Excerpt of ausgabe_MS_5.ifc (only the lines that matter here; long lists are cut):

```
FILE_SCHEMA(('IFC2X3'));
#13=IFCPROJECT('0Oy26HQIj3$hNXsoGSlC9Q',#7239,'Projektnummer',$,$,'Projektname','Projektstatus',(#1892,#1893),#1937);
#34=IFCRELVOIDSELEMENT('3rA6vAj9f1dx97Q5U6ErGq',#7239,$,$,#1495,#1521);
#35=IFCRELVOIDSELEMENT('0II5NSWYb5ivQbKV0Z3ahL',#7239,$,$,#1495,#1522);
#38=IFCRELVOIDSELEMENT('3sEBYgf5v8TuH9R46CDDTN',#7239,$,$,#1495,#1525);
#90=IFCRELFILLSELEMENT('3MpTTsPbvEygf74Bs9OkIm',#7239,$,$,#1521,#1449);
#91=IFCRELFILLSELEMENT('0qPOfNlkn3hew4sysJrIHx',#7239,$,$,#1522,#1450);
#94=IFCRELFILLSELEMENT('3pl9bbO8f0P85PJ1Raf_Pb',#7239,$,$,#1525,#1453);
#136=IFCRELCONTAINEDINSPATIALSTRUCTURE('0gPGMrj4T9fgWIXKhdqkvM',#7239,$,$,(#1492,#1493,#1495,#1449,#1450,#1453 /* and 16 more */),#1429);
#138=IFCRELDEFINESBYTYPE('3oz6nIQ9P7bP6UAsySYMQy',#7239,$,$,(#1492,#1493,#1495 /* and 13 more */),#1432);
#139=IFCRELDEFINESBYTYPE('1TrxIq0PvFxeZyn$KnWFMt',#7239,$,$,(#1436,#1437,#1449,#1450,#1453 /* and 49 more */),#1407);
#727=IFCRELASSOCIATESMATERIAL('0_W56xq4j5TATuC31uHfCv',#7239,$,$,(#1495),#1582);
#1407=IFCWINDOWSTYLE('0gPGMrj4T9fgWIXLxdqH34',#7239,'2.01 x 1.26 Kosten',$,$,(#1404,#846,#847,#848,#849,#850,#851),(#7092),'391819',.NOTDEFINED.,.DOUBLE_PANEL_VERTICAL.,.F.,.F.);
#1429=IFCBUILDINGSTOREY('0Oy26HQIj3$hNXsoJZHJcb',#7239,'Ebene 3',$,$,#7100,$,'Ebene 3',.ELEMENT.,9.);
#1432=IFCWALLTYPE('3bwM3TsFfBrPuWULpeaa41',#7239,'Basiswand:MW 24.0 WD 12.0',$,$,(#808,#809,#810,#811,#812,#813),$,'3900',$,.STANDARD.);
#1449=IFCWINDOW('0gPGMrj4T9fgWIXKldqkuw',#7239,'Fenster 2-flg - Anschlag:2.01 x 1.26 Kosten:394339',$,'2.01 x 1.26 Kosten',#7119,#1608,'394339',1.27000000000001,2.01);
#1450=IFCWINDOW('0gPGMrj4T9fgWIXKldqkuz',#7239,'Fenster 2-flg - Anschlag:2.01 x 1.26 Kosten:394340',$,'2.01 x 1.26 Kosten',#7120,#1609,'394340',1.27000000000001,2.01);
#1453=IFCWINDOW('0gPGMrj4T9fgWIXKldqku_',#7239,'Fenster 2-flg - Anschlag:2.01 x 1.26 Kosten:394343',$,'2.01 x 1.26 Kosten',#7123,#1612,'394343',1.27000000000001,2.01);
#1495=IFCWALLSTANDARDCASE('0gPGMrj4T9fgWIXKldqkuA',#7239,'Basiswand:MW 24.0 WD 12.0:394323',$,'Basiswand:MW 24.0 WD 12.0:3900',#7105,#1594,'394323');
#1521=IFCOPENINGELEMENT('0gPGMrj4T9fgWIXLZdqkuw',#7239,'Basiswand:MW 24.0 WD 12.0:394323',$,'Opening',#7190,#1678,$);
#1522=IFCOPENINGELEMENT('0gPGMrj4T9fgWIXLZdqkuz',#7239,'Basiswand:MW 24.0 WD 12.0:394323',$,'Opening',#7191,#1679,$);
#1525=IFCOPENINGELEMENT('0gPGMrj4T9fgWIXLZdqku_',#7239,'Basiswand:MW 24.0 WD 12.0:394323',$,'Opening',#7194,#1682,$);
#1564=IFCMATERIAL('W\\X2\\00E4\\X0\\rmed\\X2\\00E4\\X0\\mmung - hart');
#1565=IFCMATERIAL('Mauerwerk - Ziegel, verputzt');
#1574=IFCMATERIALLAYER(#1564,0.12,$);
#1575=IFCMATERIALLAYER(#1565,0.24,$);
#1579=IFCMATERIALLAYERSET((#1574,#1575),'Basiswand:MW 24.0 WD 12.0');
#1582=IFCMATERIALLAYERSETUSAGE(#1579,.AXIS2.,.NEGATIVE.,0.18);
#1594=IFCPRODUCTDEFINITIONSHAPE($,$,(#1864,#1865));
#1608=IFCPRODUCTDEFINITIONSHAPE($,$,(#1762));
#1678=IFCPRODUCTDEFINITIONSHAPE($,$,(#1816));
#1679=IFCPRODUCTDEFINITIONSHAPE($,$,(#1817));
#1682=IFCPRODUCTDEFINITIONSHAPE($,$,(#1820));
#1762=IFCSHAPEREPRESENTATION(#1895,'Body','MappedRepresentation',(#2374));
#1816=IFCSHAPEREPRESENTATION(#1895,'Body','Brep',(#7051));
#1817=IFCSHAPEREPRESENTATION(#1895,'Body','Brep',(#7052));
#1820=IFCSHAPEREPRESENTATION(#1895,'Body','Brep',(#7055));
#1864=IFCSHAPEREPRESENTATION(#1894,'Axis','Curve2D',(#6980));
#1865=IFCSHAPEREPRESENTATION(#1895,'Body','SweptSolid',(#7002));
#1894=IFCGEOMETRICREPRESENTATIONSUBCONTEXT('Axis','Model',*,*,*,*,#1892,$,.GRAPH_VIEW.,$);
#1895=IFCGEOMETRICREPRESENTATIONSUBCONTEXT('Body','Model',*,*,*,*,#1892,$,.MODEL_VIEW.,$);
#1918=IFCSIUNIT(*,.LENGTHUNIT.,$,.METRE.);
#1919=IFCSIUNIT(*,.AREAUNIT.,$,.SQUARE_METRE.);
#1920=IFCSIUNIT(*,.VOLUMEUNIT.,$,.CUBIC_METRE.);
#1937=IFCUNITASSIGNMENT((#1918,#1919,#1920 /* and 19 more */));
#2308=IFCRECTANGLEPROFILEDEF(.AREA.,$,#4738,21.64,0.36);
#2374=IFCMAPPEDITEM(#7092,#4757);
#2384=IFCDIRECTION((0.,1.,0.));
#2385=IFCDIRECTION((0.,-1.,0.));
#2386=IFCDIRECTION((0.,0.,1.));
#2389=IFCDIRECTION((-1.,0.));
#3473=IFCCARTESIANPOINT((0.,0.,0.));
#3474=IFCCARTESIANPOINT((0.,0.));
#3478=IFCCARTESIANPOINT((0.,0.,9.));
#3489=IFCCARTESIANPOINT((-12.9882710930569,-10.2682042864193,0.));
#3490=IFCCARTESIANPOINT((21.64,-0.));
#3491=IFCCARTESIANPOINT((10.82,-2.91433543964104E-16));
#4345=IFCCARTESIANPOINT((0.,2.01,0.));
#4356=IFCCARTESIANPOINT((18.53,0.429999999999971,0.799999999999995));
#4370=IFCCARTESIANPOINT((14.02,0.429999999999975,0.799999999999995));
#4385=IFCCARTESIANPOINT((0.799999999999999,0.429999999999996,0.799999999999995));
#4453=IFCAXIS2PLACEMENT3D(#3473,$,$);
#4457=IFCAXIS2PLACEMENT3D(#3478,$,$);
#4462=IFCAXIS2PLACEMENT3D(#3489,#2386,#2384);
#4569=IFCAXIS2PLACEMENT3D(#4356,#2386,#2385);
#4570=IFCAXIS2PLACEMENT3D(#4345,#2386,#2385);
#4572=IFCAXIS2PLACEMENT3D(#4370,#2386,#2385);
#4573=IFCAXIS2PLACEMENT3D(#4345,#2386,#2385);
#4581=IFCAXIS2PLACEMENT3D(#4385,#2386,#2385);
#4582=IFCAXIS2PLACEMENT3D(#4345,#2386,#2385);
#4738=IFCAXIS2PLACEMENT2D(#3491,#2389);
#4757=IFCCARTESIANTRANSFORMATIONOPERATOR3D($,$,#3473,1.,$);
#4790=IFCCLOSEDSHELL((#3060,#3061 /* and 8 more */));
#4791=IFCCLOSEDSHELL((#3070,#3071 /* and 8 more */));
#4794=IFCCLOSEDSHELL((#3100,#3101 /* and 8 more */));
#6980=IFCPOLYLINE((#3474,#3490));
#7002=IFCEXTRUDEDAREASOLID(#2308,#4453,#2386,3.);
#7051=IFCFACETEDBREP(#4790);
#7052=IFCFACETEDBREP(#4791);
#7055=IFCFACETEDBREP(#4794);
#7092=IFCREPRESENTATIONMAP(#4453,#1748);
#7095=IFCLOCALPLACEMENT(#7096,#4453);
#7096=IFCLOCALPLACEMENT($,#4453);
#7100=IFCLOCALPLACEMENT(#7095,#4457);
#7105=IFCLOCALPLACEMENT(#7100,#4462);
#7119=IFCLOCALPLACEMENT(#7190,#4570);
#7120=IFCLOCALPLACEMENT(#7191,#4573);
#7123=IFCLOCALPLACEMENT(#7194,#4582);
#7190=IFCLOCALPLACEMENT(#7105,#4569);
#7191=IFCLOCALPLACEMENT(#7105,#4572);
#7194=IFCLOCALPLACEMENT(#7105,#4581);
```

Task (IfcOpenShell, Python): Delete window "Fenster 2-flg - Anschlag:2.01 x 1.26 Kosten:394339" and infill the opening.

```python
import ifcopenshell
import ifcopenshell.api.feature
import ifcopenshell.api.root
import ifcopenshell.geom
import ifcopenshell.util.shape

model = ifcopenshell.open("ausgabe_MS_5.ifc")
settings = ifcopenshell.geom.settings()


def volume(element):
    """Net volume in cubic metres, openings subtracted."""
    shape = ifcopenshell.geom.create_shape(settings, element)
    return ifcopenshell.util.shape.get_volume(shape.geometry)


window = model.by_id(1449)
opening = window.FillsVoids[0].RelatingOpeningElement
wall = opening.VoidsElements[0].RelatingBuildingElement
before = volume(wall)

ifcopenshell.api.root.remove_product(model, product=window)
ifcopenshell.api.feature.remove_feature(model, feature=opening)

after = volume(wall)

print(f"wall volume {before:.3f} -> {after:.3f} m3")

model.write("ausgabe_MS_5-out.ifc")
```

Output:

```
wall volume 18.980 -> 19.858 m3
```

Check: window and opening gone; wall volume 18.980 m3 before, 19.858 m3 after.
